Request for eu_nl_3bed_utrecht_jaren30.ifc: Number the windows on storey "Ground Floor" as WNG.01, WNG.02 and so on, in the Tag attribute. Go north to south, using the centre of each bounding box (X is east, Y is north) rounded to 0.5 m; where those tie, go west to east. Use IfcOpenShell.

First a look at what the model holds.

```python
import ifcopenshell
import ifcopenshell.util.element
import ifcopenshell.util.placement

model = ifcopenshell.open("eu_nl_3bed_utrecht_jaren30.ifc")
print(model.schema)
storey = next(s for s in model.by_type("IfcBuildingStorey") if s.Name == "Ground Floor")
windows = [e for e in ifcopenshell.util.element.get_decomposition(storey) if e.is_a("IfcWindow")]
for e in sorted(windows, key=lambda e: e.id()):
    origin = ifcopenshell.util.placement.get_local_placement(e.ObjectPlacement)[:3, 3]
    print(e.id(), e.Tag, e.Name, origin.round(2) + 0.0, sep=" | ")
```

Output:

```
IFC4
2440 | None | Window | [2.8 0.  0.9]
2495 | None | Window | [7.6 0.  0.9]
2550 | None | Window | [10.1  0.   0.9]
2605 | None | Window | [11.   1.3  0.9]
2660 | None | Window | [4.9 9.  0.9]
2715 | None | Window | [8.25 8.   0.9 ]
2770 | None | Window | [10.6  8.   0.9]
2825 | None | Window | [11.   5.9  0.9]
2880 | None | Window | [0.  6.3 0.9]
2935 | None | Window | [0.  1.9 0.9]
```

```python
import ifcopenshell
import ifcopenshell.geom
import ifcopenshell.util.element
import ifcopenshell.util.shape

model = ifcopenshell.open("eu_nl_3bed_utrecht_jaren30.ifc")
settings = ifcopenshell.geom.settings()
settings.set("use-world-coords", True)


def centre(element):
    shape = ifcopenshell.geom.create_shape(settings, element)
    return ifcopenshell.util.shape.get_bbox_centroid(shape.geometry)


storey = next(s for s in model.by_type("IfcBuildingStorey") if s.Name == "Ground Floor")
windows = [e for e in ifcopenshell.util.element.get_decomposition(storey) if e.is_a("IfcWindow")]

# Insertion points can sit at a corner or the storey origin, so sort by the geometry (in metres).
centres = {e: centre(e) for e in windows}
windows.sort(key=lambda e: (-round(centres[e][1] / 0.5), centres[e][0]))

for i, e in enumerate(windows, start=1):
    number = f"WNG.{i:02d}"
    e.Tag = number
    print(e.id(), number)

model.write("eu_nl_3bed_utrecht_jaren30-out.ifc")
```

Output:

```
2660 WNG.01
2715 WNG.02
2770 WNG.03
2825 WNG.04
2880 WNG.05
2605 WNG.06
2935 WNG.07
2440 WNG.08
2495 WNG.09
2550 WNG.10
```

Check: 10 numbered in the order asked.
